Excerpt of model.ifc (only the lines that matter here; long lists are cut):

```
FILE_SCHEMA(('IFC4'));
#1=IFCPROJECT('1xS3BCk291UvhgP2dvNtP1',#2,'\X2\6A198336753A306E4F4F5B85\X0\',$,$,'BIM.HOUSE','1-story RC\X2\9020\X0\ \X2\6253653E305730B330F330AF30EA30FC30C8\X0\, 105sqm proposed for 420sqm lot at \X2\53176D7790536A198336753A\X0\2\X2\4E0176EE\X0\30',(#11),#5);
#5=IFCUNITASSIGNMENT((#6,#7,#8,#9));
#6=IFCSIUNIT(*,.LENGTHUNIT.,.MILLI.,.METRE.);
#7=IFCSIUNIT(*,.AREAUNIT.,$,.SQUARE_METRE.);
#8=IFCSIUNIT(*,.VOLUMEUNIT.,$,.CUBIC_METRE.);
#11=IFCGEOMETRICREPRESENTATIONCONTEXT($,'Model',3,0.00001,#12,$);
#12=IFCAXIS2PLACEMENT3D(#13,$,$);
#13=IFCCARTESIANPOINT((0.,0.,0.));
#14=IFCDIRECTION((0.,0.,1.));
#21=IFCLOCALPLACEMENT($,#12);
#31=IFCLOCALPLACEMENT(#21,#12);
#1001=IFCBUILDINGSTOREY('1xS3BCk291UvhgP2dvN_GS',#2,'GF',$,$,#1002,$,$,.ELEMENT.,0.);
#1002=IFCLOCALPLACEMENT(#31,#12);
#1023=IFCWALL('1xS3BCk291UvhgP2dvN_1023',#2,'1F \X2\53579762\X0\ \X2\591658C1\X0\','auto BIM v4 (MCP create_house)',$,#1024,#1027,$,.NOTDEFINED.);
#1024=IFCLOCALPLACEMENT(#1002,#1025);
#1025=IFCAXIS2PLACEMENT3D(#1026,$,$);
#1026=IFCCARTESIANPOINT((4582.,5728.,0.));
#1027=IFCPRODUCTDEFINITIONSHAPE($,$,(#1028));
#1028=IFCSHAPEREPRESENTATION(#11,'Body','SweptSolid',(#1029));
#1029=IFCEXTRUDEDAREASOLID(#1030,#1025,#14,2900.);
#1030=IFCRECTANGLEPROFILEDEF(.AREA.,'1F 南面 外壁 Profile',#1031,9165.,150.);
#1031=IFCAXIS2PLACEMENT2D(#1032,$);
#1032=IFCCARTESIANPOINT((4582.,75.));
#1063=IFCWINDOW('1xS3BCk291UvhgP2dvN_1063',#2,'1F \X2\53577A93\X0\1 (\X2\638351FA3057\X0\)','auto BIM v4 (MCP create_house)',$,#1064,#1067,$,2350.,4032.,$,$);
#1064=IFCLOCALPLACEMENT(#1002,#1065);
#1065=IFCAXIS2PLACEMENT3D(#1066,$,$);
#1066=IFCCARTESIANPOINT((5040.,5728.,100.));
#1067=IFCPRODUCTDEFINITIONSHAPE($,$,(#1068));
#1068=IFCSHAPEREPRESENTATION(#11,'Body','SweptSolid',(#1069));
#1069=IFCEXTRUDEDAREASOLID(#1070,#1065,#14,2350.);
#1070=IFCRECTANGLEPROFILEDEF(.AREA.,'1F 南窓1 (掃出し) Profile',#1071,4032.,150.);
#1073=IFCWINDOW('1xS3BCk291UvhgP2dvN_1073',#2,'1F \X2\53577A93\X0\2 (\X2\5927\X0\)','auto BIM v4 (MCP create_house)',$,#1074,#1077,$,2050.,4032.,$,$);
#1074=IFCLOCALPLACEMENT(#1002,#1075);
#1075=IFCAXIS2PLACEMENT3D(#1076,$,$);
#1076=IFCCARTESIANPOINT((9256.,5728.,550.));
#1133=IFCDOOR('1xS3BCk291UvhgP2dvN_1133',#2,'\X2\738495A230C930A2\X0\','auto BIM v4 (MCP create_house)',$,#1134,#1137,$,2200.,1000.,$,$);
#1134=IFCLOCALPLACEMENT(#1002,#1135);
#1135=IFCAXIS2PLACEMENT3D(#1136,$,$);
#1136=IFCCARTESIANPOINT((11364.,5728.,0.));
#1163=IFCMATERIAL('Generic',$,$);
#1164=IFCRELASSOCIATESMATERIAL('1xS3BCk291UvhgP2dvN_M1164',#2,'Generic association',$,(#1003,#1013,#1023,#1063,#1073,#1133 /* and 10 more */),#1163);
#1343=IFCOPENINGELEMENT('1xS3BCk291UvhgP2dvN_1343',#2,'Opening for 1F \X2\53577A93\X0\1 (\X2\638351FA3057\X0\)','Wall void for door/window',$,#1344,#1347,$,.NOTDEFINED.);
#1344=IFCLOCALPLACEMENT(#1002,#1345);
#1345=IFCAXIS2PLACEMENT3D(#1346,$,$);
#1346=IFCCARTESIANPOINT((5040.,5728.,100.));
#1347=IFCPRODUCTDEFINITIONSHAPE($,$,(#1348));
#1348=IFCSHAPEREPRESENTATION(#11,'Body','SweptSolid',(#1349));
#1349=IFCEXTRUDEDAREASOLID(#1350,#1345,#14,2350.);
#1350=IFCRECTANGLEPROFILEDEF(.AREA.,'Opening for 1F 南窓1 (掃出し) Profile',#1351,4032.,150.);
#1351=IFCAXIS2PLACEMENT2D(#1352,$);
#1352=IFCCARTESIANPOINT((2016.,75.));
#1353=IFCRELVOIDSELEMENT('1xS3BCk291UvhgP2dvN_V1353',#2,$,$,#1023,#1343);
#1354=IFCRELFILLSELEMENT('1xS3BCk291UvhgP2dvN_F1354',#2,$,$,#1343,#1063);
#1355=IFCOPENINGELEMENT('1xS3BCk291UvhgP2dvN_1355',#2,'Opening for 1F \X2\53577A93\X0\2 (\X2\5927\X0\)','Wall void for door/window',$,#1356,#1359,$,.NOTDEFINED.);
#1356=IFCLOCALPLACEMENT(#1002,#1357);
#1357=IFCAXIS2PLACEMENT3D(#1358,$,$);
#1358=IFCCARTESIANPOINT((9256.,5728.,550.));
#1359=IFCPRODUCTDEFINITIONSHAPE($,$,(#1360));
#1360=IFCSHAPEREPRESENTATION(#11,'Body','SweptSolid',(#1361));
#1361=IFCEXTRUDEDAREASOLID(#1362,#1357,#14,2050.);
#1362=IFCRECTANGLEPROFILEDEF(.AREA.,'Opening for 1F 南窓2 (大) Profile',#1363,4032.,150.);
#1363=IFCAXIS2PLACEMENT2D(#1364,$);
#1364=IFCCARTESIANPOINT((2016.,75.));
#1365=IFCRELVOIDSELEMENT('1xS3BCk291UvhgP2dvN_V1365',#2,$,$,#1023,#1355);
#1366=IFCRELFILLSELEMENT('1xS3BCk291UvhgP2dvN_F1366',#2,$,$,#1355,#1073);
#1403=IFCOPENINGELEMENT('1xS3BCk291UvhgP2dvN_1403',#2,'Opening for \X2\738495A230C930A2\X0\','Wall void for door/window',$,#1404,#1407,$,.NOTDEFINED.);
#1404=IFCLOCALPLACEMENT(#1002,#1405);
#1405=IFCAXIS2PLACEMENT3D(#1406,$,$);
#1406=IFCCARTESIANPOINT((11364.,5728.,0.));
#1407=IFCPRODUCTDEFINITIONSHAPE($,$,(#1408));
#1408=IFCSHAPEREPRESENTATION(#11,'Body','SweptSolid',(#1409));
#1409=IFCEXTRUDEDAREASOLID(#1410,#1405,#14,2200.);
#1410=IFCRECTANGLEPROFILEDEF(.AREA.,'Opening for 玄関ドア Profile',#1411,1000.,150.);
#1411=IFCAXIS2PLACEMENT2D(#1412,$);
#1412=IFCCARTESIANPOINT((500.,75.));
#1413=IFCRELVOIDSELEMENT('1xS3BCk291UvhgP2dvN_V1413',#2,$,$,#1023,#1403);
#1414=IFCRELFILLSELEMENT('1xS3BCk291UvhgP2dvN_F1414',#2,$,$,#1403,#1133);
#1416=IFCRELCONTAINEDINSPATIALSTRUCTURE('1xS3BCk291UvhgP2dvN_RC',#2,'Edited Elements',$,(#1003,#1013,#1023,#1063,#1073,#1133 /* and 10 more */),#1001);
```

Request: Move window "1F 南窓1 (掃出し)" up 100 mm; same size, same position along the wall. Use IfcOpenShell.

```python
import numpy as np
import ifcopenshell
import ifcopenshell.api.geometry
import ifcopenshell.util.placement
import ifcopenshell.util.unit

model = ifcopenshell.open("model.ifc")
unit_scale = ifcopenshell.util.unit.calculate_unit_scale(model)

window = model.by_id(1063)
opening = window.FillsVoids[0].RelatingOpeningElement
dz = 100.0

shift = np.array([0.0, 0.0, dz])
# The window is not placed relative to its opening, so move both.
for product in (opening, window):
    matrix = ifcopenshell.util.placement.get_local_placement(product.ObjectPlacement)
    matrix[:3, 3] += shift
    ifcopenshell.api.geometry.edit_object_placement(model, product=product, matrix=matrix, is_si=False)

print(f"moved by {dz * unit_scale:+.3f} m")

model.write("model-out.ifc")
```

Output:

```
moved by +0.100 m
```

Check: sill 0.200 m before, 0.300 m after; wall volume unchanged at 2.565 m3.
